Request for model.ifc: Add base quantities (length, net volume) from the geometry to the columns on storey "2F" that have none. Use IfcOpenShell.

First a look at what the model holds.

```python
import ifcopenshell
import ifcopenshell.util.element
import ifcopenshell.util.unit

model = ifcopenshell.open("model.ifc")
print(model.schema)
for unit_type in ("LENGTHUNIT", "AREAUNIT", "VOLUMEUNIT"):
    print(unit_type, ifcopenshell.util.unit.calculate_unit_scale(model, unit_type))
storey = next(s for s in model.by_type("IfcBuildingStorey") if s.Name == "2F")
columns = [e for e in ifcopenshell.util.element.get_decomposition(storey) if e.is_a("IfcColumn")]
for e in sorted(columns, key=lambda e: e.id()):
    print(e.id(), e.is_a(), e.Name, list(ifcopenshell.util.element.get_psets(e, qtos_only=True)), sep=" | ")
```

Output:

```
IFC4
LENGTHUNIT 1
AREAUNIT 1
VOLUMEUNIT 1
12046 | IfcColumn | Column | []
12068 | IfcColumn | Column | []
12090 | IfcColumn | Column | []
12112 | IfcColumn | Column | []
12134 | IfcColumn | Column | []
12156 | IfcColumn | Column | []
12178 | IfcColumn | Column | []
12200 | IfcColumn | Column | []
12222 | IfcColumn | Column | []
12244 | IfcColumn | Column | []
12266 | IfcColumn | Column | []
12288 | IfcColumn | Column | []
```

```python
import ifcopenshell
import ifcopenshell.api.pset
import ifcopenshell.geom
import ifcopenshell.util.element
import ifcopenshell.util.shape
import ifcopenshell.util.unit

model = ifcopenshell.open("model.ifc")
unit_scale = ifcopenshell.util.unit.calculate_unit_scale(model)
volume_scale = ifcopenshell.util.unit.calculate_unit_scale(model, "VOLUMEUNIT")
settings = ifcopenshell.geom.settings()

storey = next(s for s in model.by_type("IfcBuildingStorey") if s.Name == "2F")
columns = [e for e in ifcopenshell.util.element.get_decomposition(storey) if e.is_a("IfcColumn")]

for e in sorted(columns, key=lambda e: e.id()):
    if ifcopenshell.util.element.get_psets(e, qtos_only=True, should_inherit=False):
        continue
    # Geometry comes back in metres, in the element's own axes.
    shape = ifcopenshell.geom.create_shape(settings, e)
    values = {
        "Length": ifcopenshell.util.shape.get_z(shape.geometry) / unit_scale,
        "NetVolume": ifcopenshell.util.shape.get_volume(shape.geometry) / volume_scale,
    }
    qto = ifcopenshell.api.pset.add_qto(model, product=e, name="Qto_ColumnBaseQuantities")
    ifcopenshell.api.pset.edit_qto(model, qto=qto, properties=values)
    print(e.id(), {k: round(v, 3) for k, v in values.items()})

model.write("model_rev.ifc")
```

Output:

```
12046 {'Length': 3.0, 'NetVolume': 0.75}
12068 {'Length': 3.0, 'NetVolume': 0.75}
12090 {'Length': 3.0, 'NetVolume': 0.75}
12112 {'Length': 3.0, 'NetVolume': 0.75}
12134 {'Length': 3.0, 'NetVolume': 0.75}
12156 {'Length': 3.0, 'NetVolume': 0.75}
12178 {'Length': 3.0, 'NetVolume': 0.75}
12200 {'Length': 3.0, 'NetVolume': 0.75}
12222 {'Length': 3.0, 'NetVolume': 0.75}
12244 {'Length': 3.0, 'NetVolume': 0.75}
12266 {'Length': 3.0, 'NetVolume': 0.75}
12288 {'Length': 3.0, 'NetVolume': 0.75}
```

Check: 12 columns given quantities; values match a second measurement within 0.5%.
